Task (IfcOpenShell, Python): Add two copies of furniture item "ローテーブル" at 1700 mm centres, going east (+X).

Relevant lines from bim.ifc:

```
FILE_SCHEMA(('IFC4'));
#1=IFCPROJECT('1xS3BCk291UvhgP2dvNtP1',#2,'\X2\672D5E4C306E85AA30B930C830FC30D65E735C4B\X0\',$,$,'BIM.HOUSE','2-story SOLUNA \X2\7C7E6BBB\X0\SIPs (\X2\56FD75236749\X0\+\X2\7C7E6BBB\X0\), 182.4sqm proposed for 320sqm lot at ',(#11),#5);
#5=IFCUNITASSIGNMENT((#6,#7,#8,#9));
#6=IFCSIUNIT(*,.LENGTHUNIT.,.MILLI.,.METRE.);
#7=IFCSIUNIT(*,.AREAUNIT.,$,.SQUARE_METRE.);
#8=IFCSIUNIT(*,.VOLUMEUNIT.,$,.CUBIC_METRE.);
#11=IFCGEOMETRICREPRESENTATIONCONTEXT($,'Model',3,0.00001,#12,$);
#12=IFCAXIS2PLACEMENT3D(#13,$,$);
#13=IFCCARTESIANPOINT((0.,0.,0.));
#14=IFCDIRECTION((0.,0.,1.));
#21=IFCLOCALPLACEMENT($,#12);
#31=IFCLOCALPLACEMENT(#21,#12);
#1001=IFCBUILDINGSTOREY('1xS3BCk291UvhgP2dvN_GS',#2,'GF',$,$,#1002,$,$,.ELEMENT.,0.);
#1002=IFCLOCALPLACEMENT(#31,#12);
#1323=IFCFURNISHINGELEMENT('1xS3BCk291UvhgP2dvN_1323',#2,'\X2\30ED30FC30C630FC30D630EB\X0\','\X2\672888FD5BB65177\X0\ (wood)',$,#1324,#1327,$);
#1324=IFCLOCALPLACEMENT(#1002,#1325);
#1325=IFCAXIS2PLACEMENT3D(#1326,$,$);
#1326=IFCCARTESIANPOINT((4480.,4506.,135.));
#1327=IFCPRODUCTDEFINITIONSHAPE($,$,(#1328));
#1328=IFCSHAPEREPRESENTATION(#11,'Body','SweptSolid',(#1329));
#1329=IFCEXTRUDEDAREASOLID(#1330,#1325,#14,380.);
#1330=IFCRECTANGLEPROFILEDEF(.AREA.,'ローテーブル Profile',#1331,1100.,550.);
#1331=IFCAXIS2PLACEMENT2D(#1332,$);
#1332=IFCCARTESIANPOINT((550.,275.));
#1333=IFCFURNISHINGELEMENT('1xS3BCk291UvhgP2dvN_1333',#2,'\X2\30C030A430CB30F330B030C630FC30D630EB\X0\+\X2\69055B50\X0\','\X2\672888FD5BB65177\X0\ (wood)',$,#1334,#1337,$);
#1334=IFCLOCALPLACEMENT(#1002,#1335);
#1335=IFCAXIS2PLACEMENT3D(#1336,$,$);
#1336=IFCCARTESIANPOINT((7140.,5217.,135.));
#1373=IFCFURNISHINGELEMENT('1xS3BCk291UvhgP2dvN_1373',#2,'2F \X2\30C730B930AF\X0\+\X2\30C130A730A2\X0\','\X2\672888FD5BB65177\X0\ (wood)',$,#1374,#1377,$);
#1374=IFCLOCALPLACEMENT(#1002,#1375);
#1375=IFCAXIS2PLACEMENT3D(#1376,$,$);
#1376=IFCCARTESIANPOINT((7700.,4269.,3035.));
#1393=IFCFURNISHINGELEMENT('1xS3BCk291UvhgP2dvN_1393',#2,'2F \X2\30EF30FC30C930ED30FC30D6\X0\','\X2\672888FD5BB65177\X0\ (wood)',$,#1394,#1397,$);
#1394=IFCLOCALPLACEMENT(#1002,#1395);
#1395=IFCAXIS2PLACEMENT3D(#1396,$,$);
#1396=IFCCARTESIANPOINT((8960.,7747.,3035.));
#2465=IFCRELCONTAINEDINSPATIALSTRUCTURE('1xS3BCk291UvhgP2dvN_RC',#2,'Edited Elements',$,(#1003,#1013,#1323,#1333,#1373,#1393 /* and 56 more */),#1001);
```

```python
import numpy as np
import ifcopenshell
import ifcopenshell.api.geometry
import ifcopenshell.api.root
import ifcopenshell.util.element
import ifcopenshell.util.placement
import ifcopenshell.util.unit

model = ifcopenshell.open("bim.ifc")
unit_scale = ifcopenshell.util.unit.calculate_unit_scale(model)


def reuse_history(source, copy):
    """copy_class also copies each property set's owner history, people and application; keep the originals."""
    for rel in copy.IsDefinedBy:
        if rel.is_a("IfcRelDefinesByProperties") and (history := rel.RelatingPropertyDefinition.OwnerHistory):
            rel.RelatingPropertyDefinition.OwnerHistory = source.OwnerHistory
            ifcopenshell.util.element.remove_deep2(model, history)


source = model.by_guid("1xS3BCk291UvhgP2dvN_1323")
base = ifcopenshell.util.placement.get_local_placement(source.ObjectPlacement)
step = np.array([1.0, 0.0, 0.0]) * 1.7 / unit_scale

for i in range(1, 3):
    copy = ifcopenshell.api.root.copy_class(model, product=source)
    copy.Representation = ifcopenshell.util.element.copy_deep(
        model, source.Representation, exclude=["IfcGeometricRepresentationContext", "IfcRepresentationMap"]
    )
    reuse_history(source, copy)
    matrix = base.copy()
    matrix[:3, 3] += i * step
    print("added at", matrix[:3, 3].round(3) + 0.0)
    ifcopenshell.api.geometry.edit_object_placement(model, product=copy, matrix=matrix, is_si=False)

model.write("bim_updated.ifc")
```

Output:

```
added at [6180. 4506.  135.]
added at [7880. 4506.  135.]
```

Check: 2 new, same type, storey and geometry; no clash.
